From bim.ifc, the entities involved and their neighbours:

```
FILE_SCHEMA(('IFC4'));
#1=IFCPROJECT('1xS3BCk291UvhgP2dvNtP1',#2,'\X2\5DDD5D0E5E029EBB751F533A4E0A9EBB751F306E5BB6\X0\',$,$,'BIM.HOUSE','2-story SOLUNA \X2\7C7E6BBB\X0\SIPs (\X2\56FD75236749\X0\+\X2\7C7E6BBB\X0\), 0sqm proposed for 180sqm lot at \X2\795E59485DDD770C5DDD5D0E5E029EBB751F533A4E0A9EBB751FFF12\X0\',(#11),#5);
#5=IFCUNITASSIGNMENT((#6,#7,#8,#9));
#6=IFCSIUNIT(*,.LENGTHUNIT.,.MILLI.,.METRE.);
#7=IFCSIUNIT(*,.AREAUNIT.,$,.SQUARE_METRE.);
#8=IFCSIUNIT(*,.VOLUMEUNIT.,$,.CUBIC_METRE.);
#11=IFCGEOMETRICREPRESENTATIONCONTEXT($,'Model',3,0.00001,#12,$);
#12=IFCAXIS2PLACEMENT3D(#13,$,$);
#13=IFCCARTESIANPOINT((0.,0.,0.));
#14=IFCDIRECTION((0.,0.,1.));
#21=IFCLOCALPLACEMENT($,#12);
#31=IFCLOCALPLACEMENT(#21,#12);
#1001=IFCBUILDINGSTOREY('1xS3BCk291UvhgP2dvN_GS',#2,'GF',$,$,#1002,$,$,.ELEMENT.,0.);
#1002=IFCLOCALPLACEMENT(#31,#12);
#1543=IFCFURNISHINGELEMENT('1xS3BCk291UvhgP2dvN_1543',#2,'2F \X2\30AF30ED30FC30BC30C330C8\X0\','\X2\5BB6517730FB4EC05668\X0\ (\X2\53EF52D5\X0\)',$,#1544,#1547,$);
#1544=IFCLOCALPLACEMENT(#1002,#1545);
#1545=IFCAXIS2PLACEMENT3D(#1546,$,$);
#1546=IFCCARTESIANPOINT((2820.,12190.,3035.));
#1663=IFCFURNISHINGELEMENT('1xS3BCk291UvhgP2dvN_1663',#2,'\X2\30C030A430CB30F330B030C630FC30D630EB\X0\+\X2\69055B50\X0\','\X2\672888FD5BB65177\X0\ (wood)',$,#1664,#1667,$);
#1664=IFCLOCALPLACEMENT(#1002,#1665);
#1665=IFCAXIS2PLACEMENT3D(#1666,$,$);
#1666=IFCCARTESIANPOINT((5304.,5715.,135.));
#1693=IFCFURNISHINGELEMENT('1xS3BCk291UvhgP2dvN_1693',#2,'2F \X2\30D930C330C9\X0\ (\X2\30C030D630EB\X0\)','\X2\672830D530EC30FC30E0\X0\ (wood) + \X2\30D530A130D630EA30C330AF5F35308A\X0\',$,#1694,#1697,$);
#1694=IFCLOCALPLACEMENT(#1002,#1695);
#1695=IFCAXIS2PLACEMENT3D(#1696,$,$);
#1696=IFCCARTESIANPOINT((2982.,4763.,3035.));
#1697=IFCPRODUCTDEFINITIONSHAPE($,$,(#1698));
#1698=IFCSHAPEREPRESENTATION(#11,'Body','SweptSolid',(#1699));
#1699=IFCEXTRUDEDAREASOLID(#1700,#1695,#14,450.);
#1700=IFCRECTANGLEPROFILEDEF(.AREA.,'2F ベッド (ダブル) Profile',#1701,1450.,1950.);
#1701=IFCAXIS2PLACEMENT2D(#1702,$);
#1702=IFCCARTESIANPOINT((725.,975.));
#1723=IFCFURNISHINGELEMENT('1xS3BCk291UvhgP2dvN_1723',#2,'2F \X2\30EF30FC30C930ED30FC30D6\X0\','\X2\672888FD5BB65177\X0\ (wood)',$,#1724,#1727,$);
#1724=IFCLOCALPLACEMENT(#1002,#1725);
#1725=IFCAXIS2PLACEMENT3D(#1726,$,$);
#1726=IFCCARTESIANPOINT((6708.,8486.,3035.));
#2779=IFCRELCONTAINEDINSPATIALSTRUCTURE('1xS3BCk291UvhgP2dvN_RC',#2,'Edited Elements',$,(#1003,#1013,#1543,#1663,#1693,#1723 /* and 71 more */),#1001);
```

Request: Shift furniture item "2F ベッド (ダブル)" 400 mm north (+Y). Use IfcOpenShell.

```python
import ifcopenshell
import ifcopenshell.api.geometry
import ifcopenshell.util.placement
import ifcopenshell.util.unit

model = ifcopenshell.open("bim.ifc")
unit_scale = ifcopenshell.util.unit.calculate_unit_scale(model)

item = model.by_id(1693)
matrix = ifcopenshell.util.placement.get_local_placement(item.ObjectPlacement)
matrix[1, 3] += 0.4 / unit_scale
ifcopenshell.api.geometry.edit_object_placement(model, product=item, matrix=matrix, is_si=False)

print(ifcopenshell.util.placement.get_local_placement(item.ObjectPlacement).round(3) + 0.0)

model.write("bim_v2.ifc")
```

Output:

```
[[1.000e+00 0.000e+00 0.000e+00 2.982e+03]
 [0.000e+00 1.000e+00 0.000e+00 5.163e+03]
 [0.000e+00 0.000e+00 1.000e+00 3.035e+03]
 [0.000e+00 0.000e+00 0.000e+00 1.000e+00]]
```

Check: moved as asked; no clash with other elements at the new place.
